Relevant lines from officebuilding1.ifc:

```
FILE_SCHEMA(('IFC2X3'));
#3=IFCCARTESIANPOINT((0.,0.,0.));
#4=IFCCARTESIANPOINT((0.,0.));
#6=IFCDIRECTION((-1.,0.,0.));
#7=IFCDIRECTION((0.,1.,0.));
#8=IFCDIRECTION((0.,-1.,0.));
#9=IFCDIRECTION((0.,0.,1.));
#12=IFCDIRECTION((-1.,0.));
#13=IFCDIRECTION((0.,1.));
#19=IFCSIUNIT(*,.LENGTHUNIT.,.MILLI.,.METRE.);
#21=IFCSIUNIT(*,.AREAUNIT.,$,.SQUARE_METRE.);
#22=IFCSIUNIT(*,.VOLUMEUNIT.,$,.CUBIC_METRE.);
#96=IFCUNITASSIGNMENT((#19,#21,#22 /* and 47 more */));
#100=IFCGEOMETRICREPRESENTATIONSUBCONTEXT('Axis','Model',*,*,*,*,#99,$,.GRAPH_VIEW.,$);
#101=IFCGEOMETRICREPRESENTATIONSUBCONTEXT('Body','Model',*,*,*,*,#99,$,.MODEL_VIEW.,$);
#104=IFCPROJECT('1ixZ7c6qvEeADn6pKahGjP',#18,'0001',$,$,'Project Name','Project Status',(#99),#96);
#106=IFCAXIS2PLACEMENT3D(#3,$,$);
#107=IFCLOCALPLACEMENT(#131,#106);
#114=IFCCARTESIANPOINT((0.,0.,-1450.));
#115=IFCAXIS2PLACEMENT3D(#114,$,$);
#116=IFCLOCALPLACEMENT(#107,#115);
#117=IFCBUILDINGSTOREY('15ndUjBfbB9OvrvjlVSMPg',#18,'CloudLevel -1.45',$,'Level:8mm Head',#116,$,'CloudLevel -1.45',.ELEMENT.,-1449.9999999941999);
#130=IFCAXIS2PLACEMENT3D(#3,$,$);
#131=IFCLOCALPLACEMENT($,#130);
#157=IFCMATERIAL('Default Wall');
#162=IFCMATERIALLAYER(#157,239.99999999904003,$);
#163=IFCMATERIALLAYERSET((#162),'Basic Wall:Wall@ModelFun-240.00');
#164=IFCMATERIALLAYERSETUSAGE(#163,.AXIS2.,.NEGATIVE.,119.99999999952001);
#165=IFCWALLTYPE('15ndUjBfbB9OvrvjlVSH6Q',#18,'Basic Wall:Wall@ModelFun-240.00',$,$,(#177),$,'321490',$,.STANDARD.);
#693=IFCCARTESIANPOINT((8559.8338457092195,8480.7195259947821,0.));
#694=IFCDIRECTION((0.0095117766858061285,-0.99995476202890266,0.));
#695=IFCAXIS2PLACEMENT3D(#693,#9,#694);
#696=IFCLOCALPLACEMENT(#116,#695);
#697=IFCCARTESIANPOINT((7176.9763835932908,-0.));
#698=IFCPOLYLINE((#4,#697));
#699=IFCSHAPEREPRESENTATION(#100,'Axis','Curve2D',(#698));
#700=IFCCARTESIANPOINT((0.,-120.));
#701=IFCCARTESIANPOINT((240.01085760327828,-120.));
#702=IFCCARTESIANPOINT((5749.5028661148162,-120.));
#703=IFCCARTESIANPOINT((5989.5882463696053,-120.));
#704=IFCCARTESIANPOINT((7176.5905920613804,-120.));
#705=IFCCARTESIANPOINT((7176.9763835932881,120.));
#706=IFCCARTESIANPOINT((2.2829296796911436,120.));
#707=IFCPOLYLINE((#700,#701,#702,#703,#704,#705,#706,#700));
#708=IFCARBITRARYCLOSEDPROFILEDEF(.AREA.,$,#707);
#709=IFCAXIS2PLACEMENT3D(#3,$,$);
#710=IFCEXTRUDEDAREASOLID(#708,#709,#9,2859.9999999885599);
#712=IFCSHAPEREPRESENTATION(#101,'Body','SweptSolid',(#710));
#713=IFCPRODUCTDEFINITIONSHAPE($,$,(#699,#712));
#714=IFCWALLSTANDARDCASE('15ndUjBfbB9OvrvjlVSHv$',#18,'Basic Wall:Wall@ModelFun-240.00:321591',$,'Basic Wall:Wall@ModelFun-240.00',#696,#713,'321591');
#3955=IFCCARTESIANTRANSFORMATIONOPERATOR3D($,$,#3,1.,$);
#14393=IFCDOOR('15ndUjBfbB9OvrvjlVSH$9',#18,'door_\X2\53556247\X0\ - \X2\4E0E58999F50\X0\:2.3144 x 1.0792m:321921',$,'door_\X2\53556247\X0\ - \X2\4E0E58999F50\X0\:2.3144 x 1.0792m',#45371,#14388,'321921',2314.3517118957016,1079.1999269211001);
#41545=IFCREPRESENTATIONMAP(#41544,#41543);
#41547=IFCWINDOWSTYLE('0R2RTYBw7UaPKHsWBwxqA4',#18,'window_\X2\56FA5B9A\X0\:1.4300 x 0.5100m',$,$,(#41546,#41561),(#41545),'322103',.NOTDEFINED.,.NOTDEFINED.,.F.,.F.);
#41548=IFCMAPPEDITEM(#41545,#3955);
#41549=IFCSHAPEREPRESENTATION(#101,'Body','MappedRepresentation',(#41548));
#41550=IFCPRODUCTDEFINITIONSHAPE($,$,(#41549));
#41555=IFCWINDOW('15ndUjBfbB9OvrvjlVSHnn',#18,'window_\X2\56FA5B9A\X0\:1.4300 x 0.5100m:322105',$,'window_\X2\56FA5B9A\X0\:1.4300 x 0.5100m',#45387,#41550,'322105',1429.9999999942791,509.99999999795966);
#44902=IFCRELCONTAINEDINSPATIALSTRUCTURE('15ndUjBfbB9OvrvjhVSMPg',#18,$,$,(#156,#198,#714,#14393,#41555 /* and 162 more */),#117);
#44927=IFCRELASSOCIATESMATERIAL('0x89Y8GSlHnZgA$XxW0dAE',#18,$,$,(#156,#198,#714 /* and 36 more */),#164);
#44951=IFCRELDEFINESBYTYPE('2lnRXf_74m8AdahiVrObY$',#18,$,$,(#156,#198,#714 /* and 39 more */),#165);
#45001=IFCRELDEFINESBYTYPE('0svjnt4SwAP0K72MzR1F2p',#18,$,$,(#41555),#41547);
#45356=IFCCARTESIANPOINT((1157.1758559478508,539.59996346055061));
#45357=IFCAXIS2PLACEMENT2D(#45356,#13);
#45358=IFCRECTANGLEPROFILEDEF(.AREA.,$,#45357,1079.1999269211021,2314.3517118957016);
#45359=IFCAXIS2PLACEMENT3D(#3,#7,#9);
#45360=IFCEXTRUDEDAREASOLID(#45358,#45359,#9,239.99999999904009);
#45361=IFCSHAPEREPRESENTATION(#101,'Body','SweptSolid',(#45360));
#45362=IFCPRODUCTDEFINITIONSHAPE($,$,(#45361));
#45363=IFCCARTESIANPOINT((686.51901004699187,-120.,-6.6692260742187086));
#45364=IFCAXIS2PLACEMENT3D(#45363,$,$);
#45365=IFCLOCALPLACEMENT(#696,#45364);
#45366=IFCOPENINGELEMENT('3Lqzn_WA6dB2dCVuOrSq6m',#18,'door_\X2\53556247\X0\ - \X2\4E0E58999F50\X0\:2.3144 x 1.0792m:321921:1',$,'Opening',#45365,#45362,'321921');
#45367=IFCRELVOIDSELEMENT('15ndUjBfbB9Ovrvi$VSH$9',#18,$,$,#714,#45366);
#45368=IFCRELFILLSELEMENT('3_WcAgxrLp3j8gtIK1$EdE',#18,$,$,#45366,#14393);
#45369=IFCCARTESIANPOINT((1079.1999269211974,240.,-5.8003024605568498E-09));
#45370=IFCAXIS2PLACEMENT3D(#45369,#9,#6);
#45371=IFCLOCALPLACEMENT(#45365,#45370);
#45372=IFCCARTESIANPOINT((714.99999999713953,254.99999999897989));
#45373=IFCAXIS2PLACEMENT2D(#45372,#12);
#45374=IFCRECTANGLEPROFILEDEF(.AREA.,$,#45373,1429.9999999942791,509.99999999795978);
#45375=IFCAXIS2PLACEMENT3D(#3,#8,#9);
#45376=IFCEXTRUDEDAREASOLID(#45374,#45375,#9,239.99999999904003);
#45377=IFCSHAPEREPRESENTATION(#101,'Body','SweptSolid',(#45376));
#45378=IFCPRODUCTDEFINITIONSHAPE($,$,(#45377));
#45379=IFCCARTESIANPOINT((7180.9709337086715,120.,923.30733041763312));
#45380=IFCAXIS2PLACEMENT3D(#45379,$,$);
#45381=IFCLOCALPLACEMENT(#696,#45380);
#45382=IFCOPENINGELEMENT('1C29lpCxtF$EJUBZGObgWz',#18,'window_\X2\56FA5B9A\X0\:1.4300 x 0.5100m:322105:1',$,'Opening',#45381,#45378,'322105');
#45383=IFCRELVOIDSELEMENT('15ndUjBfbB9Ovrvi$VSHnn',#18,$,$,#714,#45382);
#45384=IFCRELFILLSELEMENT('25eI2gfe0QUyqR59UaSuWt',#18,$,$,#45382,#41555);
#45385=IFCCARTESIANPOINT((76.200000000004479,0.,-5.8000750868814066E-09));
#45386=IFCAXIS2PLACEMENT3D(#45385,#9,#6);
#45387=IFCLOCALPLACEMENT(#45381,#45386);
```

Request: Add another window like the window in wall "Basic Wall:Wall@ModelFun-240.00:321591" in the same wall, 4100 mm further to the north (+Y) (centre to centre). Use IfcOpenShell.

```python
import ifcopenshell
import ifcopenshell.api.feature
import ifcopenshell.api.geometry
import ifcopenshell.api.root
import ifcopenshell.geom
import ifcopenshell.util.element
import ifcopenshell.util.placement
import ifcopenshell.util.shape
import ifcopenshell.util.unit

model = ifcopenshell.open("officebuilding1.ifc")
unit_scale = ifcopenshell.util.unit.calculate_unit_scale(model)
settings = ifcopenshell.geom.settings()


def volume(element):
    """Net volume in cubic metres, openings subtracted."""
    shape = ifcopenshell.geom.create_shape(settings, element)
    return ifcopenshell.util.shape.get_volume(shape.geometry)


def reuse_history(source, copy):
    """copy_class also copies each property set's owner history, people and application; keep the originals."""
    for rel in copy.IsDefinedBy:
        if rel.is_a("IfcRelDefinesByProperties") and (history := rel.RelatingPropertyDefinition.OwnerHistory):
            rel.RelatingPropertyDefinition.OwnerHistory = source.OwnerHistory
            ifcopenshell.util.element.remove_deep2(model, history)


window = model.by_guid("15ndUjBfbB9OvrvjlVSHnn")
opening = window.FillsVoids[0].RelatingOpeningElement
wall = opening.VoidsElements[0].RelatingBuildingElement
before = volume(wall)
shift = ifcopenshell.util.placement.get_local_placement(wall.ObjectPlacement)[:3, 0] * -4.1 / unit_scale

# copy_class copies the void relationship, type, container and properties, but no geometry.
new_opening = ifcopenshell.api.root.copy_class(model, product=opening)
new_opening.Representation = ifcopenshell.util.element.copy_deep(
    model, opening.Representation, exclude=["IfcGeometricRepresentationContext", "IfcRepresentationMap"]
)
new_opening.Name = "window_固定:1.4300 x 0.5100m"
new_opening.Tag = None
new_window = ifcopenshell.api.root.copy_class(model, product=window)
new_window.Representation = ifcopenshell.util.element.copy_deep(
    model, window.Representation, exclude=["IfcGeometricRepresentationContext", "IfcRepresentationMap"]
)
new_window.Name = "window_固定:1.4300 x 0.5100m"
new_window.Tag = None
reuse_history(window, new_window)
fills = ifcopenshell.api.feature.add_filling(model, opening=new_opening, element=new_window)
fills.OwnerHistory = new_window.OwnerHistory  # required in IFC2X3

for old, new in ((opening, new_opening), (window, new_window)):
    matrix = ifcopenshell.util.placement.get_local_placement(old.ObjectPlacement)
    matrix[:3, 3] += shift
    ifcopenshell.api.geometry.edit_object_placement(model, product=new, matrix=matrix, is_si=False)

after = volume(wall)

print(f"wall volume {before:.3f} -> {after:.3f} m3")

model.write("officebuilding1_v2.ifc")
```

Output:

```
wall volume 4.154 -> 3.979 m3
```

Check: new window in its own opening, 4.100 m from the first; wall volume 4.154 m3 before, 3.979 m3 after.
